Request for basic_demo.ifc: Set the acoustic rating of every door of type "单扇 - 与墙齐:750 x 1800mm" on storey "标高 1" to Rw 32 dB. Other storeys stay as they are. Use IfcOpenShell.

First a look at what the model holds.

```python
import ifcopenshell
import ifcopenshell.util.element

model = ifcopenshell.open("basic_demo.ifc")
print(model.schema)
storey = next(s for s in model.by_type("IfcBuildingStorey") if s.Name == "标高 1")
doors = [e for e in ifcopenshell.util.element.get_decomposition(storey) if e.is_a("IfcDoor")]
seen = {}
for e in doors:
    element_type = ifcopenshell.util.element.get_type(e)
    key = (element_type.Name if element_type != e and element_type else None, ifcopenshell.util.element.get_pset(e, "Pset_DoorCommon", "AcousticRating"))
    seen[key] = seen.get(key, 0) + 1
for (name, value), count in sorted(seen.items(), key=str):
    print(count, "x", name, "|", value)
```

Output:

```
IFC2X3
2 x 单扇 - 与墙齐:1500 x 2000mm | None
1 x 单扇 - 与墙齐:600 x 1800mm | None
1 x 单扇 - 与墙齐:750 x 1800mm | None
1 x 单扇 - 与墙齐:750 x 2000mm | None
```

```python
import ifcopenshell
import ifcopenshell.api.pset
import ifcopenshell.util.element

model = ifcopenshell.open("basic_demo.ifc")

storey = next(s for s in model.by_type("IfcBuildingStorey") if s.Name == "标高 1")
doors = [e for e in ifcopenshell.util.element.get_decomposition(storey) if e.is_a("IfcDoor")]

count = 0
for e in doors:
    element_type = ifcopenshell.util.element.get_type(e)
    if element_type in (None, e) or element_type.Name != "单扇 - 与墙齐:750 x 1800mm":
        continue
    # add_pset returns the element's existing set when there is one.
    pset = ifcopenshell.api.pset.add_pset(model, product=e, name="Pset_DoorCommon")
    ifcopenshell.api.pset.edit_pset(model, pset=pset, properties={"AcousticRating": "Rw 32 dB"})
    count += 1

print(count, "doors updated")

model.write("basic_demo_updated.ifc")
```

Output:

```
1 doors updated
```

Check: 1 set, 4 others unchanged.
